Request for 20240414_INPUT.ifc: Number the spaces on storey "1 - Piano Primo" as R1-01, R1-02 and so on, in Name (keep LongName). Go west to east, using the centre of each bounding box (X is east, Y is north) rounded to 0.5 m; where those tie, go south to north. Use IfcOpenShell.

First a look at what the model holds.

```python
import ifcopenshell
import ifcopenshell.util.element
import ifcopenshell.util.placement

model = ifcopenshell.open("20240414_INPUT.ifc")
print(model.schema)
storey = next(s for s in model.by_type("IfcBuildingStorey") if s.Name == "1 - Piano Primo")
spaces = [e for e in ifcopenshell.util.element.get_decomposition(storey) if e.is_a("IfcSpace")]
for e in sorted(spaces, key=lambda e: e.id()):
    origin = ifcopenshell.util.placement.get_local_placement(e.ObjectPlacement)[:3, 3]
    print(e.id(), e.Name, e.LongName, origin.round(2) + 0.0, sep=" | ")
```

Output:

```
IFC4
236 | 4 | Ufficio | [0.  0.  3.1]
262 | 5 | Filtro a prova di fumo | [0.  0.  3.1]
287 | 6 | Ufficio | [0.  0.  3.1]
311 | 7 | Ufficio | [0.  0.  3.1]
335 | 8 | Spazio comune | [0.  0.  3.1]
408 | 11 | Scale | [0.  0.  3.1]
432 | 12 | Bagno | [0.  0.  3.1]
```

```python
import ifcopenshell
import ifcopenshell.geom
import ifcopenshell.util.element
import ifcopenshell.util.shape

model = ifcopenshell.open("20240414_INPUT.ifc")
settings = ifcopenshell.geom.settings()
settings.set("use-world-coords", True)


def centre(element):
    shape = ifcopenshell.geom.create_shape(settings, element)
    return ifcopenshell.util.shape.get_bbox_centroid(shape.geometry)


storey = next(s for s in model.by_type("IfcBuildingStorey") if s.Name == "1 - Piano Primo")
spaces = [e for e in ifcopenshell.util.element.get_decomposition(storey) if e.is_a("IfcSpace")]

# Insertion points can sit at a corner or the storey origin, so sort by the geometry (in metres).
centres = {e: centre(e) for e in spaces}
spaces.sort(key=lambda e: (round(centres[e][0] / 0.5), centres[e][1]))

for i, e in enumerate(spaces, start=1):
    number = f"R1-{i:02d}"
    e.Name = number
    print(e.id(), number)

model.write("20240414_INPUT_edited.ifc")
```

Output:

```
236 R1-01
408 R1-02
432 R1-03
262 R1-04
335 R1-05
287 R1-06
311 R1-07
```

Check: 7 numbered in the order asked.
